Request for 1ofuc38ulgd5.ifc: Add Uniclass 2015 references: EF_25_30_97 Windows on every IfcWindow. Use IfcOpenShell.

First a look at what the model holds.

```python
import ifcopenshell

model = ifcopenshell.open("1ofuc38ulgd5.ifc")
print(model.schema)
print("classifications:", [c.Name for c in model.by_type("IfcClassification")])
for ifc_class in ("IfcDoor", "IfcRoof", "IfcStair", "IfcWall", "IfcWindow"):
    print(ifc_class, len(model.by_type(ifc_class)))
```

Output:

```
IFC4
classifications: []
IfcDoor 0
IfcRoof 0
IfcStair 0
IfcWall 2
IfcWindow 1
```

```python
import ifcopenshell
import ifcopenshell.api.classification

model = ifcopenshell.open("1ofuc38ulgd5.ifc")

system = ifcopenshell.api.classification.add_classification(model, classification="Uniclass 2015")

codes = {
    "IfcWindow": ("EF_25_30_97", "Windows"),
}
for ifc_class, (code, name) in codes.items():
    products = model.by_type(ifc_class)
    ifcopenshell.api.classification.add_reference(
        model, products=products, classification=system, identification=code, name=name
    )
    print(code, len(products))

model.write("1ofuc38ulgd5_rev.ifc")
```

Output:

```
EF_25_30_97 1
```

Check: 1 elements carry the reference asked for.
